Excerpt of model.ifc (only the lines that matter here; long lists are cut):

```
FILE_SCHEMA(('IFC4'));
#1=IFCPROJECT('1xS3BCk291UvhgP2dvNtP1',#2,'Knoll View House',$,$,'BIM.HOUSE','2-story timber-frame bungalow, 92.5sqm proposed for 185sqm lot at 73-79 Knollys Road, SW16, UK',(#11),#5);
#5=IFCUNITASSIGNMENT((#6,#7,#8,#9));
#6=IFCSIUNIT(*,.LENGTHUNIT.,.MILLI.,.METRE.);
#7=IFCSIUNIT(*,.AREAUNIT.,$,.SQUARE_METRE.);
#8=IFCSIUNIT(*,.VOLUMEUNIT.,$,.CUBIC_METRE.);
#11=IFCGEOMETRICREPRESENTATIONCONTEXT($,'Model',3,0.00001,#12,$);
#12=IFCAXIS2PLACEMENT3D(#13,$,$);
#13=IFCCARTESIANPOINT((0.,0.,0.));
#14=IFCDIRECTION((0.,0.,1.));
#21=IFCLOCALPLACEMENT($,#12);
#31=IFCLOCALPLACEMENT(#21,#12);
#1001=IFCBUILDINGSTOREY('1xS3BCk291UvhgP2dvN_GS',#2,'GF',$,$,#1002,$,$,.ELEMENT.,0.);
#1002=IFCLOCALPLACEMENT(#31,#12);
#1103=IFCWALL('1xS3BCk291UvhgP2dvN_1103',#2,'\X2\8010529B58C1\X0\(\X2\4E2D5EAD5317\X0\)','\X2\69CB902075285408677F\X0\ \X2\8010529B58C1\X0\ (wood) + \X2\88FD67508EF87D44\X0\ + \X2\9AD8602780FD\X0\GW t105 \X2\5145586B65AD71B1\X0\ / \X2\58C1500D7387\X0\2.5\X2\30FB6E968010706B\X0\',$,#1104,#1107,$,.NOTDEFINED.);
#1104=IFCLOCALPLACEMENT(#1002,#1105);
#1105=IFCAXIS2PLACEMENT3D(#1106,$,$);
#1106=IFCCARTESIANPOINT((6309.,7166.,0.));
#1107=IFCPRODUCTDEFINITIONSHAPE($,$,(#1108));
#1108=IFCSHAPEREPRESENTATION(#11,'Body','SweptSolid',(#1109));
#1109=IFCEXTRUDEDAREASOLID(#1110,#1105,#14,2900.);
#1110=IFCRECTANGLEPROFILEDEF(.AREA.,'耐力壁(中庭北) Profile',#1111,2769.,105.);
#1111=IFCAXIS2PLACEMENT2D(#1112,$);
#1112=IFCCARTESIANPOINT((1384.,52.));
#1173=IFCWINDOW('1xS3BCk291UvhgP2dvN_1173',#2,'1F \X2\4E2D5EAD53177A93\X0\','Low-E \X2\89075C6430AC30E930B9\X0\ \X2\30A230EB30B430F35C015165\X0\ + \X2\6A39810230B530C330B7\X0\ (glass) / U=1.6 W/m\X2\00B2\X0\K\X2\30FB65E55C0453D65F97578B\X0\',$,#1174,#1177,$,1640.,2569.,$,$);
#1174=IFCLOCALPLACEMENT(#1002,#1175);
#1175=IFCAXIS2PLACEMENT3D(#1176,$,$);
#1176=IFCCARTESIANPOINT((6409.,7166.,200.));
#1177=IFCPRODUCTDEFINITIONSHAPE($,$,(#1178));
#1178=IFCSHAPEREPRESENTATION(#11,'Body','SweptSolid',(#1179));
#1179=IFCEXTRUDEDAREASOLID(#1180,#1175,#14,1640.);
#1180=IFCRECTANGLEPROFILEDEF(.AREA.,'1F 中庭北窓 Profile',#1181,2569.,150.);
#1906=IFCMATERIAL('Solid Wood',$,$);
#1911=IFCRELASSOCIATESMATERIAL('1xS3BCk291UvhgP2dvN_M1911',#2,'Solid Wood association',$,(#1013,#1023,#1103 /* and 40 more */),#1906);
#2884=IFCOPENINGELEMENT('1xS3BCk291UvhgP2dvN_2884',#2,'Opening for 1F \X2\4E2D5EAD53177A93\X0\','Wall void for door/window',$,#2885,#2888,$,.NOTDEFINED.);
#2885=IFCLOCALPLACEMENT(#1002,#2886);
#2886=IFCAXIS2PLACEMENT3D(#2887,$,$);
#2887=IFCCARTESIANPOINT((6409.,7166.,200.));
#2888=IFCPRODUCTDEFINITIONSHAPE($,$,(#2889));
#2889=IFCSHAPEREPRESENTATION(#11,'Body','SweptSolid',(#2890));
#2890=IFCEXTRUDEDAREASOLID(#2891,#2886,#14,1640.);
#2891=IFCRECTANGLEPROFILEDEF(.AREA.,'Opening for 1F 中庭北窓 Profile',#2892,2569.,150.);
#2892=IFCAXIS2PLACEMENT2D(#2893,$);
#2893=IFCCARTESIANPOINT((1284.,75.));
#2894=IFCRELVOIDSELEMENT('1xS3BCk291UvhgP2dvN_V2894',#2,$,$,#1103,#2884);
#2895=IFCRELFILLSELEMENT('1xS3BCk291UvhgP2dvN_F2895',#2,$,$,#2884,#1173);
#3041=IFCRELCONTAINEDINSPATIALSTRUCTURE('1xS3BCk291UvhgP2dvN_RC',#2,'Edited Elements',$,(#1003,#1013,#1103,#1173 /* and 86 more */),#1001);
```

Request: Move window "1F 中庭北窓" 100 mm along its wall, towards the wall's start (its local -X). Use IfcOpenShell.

```python
import ifcopenshell
import ifcopenshell.api.geometry
import ifcopenshell.util.placement
import ifcopenshell.util.unit

model = ifcopenshell.open("model.ifc")
unit_scale = ifcopenshell.util.unit.calculate_unit_scale(model)

window = model.by_guid("1xS3BCk291UvhgP2dvN_1173")
opening = window.FillsVoids[0].RelatingOpeningElement
wall = opening.VoidsElements[0].RelatingBuildingElement

wall_matrix = ifcopenshell.util.placement.get_local_placement(wall.ObjectPlacement)
shift = wall_matrix[:3, 0] * -0.1 / unit_scale
before = ifcopenshell.util.placement.get_local_placement(window.ObjectPlacement)[:3, 3].copy()

# The window is not placed relative to its opening, so move both.
for product in (opening, window):
    matrix = ifcopenshell.util.placement.get_local_placement(product.ObjectPlacement)
    matrix[:3, 3] += shift
    ifcopenshell.api.geometry.edit_object_placement(model, product=product, matrix=matrix, is_si=False)

after = ifcopenshell.util.placement.get_local_placement(window.ObjectPlacement)[:3, 3]
print("window moved by", (after - before).round(3) + 0.0)

model.write("model-out.ifc")
```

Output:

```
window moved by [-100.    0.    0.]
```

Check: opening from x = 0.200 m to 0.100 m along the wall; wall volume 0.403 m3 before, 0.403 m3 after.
